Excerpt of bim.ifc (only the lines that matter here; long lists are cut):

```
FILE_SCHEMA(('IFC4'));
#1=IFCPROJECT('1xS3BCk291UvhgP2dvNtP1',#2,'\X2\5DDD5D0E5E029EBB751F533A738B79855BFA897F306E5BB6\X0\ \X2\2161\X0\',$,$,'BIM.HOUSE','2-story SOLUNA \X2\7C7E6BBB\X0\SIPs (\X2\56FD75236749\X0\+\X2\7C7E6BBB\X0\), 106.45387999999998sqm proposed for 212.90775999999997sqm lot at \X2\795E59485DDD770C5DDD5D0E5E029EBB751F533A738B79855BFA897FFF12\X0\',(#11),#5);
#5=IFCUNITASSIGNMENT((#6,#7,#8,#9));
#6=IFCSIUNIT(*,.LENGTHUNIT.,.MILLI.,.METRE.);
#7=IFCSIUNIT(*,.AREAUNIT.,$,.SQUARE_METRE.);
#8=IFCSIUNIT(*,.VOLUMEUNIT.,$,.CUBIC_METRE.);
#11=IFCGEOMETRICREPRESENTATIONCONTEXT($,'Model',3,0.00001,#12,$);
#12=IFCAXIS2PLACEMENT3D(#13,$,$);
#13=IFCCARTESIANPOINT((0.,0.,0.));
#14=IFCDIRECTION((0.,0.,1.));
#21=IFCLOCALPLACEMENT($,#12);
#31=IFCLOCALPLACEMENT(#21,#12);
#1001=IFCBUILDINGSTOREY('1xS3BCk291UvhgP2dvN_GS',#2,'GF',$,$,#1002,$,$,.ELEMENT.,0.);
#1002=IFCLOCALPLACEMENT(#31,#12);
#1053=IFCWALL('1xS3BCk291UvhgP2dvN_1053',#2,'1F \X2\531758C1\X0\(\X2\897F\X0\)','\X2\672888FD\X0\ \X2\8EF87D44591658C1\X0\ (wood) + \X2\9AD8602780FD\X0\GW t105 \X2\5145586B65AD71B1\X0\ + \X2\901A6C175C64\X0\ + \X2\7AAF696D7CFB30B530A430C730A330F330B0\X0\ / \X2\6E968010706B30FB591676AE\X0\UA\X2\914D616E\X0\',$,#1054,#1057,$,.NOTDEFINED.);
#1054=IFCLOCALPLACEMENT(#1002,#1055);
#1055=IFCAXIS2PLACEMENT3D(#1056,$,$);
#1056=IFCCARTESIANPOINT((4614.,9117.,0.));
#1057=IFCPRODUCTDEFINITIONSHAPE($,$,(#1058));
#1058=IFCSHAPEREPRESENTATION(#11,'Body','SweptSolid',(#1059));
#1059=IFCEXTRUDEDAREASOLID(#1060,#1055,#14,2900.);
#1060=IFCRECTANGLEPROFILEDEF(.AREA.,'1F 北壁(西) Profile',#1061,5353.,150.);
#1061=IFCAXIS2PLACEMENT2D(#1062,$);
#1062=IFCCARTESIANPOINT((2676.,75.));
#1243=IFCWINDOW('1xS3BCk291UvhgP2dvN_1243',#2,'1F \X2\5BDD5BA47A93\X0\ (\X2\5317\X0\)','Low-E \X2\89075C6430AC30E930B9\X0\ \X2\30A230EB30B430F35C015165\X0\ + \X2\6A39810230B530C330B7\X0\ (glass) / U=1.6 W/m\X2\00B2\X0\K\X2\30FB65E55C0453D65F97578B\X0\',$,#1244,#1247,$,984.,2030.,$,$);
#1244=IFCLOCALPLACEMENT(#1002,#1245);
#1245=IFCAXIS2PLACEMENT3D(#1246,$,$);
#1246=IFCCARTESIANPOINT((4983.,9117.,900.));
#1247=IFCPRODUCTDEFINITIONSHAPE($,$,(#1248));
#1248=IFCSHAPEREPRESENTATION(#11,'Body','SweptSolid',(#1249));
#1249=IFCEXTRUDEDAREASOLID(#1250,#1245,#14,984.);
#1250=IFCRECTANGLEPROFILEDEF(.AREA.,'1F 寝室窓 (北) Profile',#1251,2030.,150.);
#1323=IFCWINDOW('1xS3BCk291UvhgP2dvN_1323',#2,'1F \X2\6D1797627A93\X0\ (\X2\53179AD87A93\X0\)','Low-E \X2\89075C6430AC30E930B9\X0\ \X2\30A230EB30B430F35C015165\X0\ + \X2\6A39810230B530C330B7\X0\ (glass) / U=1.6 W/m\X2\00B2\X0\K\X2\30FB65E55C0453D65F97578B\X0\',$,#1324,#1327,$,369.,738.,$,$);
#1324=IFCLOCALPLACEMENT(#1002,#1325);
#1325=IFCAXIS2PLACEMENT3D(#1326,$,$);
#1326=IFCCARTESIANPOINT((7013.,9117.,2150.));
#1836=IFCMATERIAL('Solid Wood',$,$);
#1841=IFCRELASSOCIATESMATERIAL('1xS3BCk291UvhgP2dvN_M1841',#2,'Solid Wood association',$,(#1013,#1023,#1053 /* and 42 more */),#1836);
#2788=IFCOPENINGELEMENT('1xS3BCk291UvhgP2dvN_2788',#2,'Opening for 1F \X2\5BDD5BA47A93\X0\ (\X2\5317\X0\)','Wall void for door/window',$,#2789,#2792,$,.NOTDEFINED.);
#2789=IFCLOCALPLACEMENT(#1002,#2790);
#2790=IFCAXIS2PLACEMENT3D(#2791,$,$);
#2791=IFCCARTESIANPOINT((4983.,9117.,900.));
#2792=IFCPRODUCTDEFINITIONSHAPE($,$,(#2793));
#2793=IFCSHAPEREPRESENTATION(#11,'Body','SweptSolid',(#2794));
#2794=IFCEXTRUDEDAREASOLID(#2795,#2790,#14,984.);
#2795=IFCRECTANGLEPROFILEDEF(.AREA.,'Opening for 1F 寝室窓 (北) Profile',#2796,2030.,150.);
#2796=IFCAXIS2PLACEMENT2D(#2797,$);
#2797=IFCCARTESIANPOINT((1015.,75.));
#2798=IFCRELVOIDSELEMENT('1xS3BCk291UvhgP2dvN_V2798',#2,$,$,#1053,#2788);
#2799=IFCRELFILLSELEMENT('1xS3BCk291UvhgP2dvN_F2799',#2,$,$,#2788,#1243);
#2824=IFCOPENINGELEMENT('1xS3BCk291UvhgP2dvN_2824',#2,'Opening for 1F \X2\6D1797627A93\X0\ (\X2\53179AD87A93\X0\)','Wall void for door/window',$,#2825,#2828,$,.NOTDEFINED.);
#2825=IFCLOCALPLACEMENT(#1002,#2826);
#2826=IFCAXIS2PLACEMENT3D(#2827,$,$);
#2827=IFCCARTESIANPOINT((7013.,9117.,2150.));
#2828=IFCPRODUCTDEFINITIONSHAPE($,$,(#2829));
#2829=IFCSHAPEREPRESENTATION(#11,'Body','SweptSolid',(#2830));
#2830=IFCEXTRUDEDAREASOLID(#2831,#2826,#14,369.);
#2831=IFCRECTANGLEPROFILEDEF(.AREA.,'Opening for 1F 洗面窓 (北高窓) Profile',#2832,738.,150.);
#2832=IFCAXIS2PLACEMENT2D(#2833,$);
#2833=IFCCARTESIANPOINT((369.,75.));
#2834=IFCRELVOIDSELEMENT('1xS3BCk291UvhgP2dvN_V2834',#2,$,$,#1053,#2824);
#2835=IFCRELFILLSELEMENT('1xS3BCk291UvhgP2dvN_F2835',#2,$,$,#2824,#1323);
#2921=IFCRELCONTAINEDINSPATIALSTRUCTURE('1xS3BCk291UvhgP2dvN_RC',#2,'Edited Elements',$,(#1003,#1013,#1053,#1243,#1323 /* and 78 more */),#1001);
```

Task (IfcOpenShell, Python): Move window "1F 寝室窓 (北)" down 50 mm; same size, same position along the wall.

```python
import numpy as np
import ifcopenshell
import ifcopenshell.api.geometry
import ifcopenshell.util.placement
import ifcopenshell.util.unit

model = ifcopenshell.open("bim.ifc")
unit_scale = ifcopenshell.util.unit.calculate_unit_scale(model)

window = model.by_guid("1xS3BCk291UvhgP2dvN_1243")
opening = window.FillsVoids[0].RelatingOpeningElement
dz = -0.05 / unit_scale

shift = np.array([0.0, 0.0, dz])
# The window is not placed relative to its opening, so move both.
for product in (opening, window):
    matrix = ifcopenshell.util.placement.get_local_placement(product.ObjectPlacement)
    matrix[:3, 3] += shift
    ifcopenshell.api.geometry.edit_object_placement(model, product=product, matrix=matrix, is_si=False)

print(f"moved by {dz * unit_scale:+.3f} m")

model.write("bim_edited.ifc")
```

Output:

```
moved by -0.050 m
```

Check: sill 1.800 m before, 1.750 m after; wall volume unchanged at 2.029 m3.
